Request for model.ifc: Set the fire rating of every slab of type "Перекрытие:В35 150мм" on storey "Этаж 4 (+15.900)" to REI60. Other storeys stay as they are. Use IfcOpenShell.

First a look at what the model holds.

```python
import ifcopenshell
import ifcopenshell.util.element

model = ifcopenshell.open("model.ifc")
print(model.schema)
storey = next(s for s in model.by_type("IfcBuildingStorey") if s.Name == "Этаж 4 (+15.900)")
slabs = [e for e in ifcopenshell.util.element.get_decomposition(storey) if e.is_a("IfcSlab")]
seen = {}
for e in slabs:
    element_type = ifcopenshell.util.element.get_type(e)
    key = (element_type.Name if element_type != e and element_type else None, ifcopenshell.util.element.get_pset(e, "Pset_SlabCommon", "FireRating"))
    seen[key] = seen.get(key, 0) + 1
for (name, value), count in sorted(seen.items(), key=str):
    print(count, "x", name, "|", value)
```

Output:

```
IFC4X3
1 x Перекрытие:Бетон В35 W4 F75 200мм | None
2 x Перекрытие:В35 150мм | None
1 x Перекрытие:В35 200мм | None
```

```python
import ifcopenshell
import ifcopenshell.api.pset
import ifcopenshell.util.element

model = ifcopenshell.open("model.ifc")

storey = next(s for s in model.by_type("IfcBuildingStorey") if s.Name == "Этаж 4 (+15.900)")
slabs = [e for e in ifcopenshell.util.element.get_decomposition(storey) if e.is_a("IfcSlab")]

count = 0
for e in slabs:
    element_type = ifcopenshell.util.element.get_type(e)
    if element_type in (None, e) or element_type.Name != "Перекрытие:В35 150мм":
        continue
    # add_pset returns the element's existing set when there is one.
    pset = ifcopenshell.api.pset.add_pset(model, product=e, name="Pset_SlabCommon")
    ifcopenshell.api.pset.edit_pset(model, pset=pset, properties={"FireRating": "REI60"})
    count += 1

print(count, "slabs updated")

model.write("model_updated.ifc")
```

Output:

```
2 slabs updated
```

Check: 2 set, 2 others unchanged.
